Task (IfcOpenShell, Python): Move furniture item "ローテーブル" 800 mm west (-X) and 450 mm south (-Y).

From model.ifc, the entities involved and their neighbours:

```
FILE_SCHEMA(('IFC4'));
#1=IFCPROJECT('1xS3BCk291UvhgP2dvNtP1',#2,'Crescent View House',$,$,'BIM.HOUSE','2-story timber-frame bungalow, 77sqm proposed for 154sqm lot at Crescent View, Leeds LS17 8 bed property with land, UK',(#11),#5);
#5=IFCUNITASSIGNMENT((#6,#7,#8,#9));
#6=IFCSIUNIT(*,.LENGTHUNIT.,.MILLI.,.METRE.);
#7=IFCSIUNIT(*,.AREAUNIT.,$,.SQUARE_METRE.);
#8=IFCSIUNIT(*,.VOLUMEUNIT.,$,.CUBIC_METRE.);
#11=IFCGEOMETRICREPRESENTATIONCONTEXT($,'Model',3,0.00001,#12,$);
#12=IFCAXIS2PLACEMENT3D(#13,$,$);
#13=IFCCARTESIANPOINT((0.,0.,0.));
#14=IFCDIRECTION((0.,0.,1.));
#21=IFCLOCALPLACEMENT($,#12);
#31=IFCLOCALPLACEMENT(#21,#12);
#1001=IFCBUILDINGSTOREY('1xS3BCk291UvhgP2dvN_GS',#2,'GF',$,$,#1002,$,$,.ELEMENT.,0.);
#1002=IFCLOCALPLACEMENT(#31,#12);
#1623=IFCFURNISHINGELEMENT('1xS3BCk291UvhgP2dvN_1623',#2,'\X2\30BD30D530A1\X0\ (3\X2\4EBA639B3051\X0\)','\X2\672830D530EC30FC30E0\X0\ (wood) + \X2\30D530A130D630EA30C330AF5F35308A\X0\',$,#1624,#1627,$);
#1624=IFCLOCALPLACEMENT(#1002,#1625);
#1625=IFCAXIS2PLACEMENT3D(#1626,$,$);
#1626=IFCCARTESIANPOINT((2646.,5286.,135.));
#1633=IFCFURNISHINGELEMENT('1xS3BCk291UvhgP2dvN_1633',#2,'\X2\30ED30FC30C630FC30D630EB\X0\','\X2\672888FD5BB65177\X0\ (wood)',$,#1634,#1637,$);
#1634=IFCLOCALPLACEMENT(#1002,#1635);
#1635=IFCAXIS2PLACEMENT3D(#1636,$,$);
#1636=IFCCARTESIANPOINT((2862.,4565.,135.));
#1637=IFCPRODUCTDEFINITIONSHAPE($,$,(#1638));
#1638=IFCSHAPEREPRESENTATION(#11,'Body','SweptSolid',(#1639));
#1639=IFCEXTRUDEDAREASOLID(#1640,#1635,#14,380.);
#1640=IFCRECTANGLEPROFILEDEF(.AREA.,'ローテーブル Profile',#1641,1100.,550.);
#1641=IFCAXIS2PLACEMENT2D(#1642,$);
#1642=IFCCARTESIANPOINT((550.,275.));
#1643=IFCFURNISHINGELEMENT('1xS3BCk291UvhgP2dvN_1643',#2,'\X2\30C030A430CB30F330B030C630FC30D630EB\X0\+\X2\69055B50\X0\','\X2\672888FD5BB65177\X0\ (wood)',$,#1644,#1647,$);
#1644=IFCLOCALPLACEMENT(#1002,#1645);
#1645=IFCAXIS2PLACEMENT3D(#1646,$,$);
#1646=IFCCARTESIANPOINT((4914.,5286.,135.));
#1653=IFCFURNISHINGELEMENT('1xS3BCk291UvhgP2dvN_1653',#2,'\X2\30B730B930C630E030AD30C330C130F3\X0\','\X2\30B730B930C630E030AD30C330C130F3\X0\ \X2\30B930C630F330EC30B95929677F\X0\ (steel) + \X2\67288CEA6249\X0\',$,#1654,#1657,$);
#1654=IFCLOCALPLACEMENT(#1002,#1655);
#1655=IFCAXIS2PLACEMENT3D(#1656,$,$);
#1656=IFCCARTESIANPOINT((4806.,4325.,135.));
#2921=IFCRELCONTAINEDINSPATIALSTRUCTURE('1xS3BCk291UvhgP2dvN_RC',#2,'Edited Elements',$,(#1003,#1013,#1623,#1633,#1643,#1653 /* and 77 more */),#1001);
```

```python
import ifcopenshell
import ifcopenshell.api.geometry
import ifcopenshell.util.placement
import ifcopenshell.util.unit

model = ifcopenshell.open("model.ifc")
unit_scale = ifcopenshell.util.unit.calculate_unit_scale(model)

item = model.by_guid("1xS3BCk291UvhgP2dvN_1633")
matrix = ifcopenshell.util.placement.get_local_placement(item.ObjectPlacement)
matrix[0, 3] -= 0.8 / unit_scale
matrix[1, 3] -= 0.45 / unit_scale
ifcopenshell.api.geometry.edit_object_placement(model, product=item, matrix=matrix, is_si=False)

print(ifcopenshell.util.placement.get_local_placement(item.ObjectPlacement).round(3) + 0.0)

model.write("model_rev.ifc")
```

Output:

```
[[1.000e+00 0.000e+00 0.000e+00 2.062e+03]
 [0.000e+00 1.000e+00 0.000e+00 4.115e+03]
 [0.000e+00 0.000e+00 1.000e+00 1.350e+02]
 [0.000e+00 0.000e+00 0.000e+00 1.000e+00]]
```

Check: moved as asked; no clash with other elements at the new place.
